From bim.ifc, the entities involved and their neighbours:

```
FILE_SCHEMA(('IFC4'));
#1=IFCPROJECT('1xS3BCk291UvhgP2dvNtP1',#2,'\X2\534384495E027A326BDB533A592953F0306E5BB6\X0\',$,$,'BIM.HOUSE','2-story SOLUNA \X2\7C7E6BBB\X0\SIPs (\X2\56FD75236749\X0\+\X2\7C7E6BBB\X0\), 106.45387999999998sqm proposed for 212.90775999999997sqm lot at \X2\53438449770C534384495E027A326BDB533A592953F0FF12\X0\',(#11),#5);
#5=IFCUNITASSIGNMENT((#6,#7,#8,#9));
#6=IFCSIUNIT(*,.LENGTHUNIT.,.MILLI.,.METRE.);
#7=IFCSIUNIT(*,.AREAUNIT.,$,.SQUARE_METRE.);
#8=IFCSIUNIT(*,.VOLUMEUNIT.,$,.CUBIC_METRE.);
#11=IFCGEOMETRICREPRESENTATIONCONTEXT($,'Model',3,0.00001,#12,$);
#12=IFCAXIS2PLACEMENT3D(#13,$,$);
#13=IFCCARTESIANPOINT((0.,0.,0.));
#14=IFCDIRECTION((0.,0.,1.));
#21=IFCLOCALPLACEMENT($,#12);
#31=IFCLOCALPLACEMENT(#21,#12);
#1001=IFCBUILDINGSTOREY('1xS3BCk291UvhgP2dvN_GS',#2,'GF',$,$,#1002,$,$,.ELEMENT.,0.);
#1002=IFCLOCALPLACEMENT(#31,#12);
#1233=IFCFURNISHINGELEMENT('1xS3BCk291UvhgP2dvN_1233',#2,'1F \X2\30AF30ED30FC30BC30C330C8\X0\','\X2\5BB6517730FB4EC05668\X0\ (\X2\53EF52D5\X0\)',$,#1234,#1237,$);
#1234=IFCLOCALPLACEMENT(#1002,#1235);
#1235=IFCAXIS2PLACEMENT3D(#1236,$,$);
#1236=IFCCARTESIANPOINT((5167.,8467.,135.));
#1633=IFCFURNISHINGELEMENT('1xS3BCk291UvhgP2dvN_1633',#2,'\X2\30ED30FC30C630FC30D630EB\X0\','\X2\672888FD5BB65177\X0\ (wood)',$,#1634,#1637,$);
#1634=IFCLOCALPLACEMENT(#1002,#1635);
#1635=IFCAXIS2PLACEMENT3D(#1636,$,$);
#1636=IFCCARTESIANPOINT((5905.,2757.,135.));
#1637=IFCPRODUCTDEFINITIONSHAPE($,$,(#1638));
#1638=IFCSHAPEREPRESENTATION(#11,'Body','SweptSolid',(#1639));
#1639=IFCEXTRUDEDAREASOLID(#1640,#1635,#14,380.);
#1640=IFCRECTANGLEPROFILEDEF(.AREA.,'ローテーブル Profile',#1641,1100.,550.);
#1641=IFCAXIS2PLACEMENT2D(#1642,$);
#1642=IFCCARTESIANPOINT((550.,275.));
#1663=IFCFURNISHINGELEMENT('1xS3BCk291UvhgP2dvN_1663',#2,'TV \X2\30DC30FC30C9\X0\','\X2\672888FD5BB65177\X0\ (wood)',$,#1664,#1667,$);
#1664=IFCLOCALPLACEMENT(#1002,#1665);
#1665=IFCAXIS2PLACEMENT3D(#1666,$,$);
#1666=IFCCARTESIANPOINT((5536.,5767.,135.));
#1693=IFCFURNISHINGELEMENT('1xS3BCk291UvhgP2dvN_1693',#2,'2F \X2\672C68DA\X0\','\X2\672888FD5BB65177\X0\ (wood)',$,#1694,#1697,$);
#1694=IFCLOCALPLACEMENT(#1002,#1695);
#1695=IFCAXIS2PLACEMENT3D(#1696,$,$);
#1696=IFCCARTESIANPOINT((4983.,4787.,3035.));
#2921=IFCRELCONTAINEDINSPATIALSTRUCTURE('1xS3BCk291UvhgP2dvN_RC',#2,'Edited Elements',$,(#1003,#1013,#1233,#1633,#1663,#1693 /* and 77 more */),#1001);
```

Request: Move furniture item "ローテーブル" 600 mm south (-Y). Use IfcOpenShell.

```python
import ifcopenshell
import ifcopenshell.api.geometry
import ifcopenshell.util.placement
import ifcopenshell.util.unit

model = ifcopenshell.open("bim.ifc")
unit_scale = ifcopenshell.util.unit.calculate_unit_scale(model)

item = model.by_guid("1xS3BCk291UvhgP2dvN_1633")
matrix = ifcopenshell.util.placement.get_local_placement(item.ObjectPlacement)
matrix[1, 3] -= 0.6 / unit_scale
ifcopenshell.api.geometry.edit_object_placement(model, product=item, matrix=matrix, is_si=False)

print(ifcopenshell.util.placement.get_local_placement(item.ObjectPlacement).round(3) + 0.0)

model.write("bim_updated.ifc")
```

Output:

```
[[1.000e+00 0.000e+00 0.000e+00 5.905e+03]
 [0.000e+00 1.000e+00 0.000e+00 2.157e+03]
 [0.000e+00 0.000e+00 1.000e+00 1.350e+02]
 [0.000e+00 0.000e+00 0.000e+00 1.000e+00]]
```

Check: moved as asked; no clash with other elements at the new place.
